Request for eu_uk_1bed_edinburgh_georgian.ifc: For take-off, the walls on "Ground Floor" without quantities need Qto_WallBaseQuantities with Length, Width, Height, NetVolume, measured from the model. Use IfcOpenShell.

First a look at what the model holds.

```python
import ifcopenshell
import ifcopenshell.util.element
import ifcopenshell.util.unit

model = ifcopenshell.open("eu_uk_1bed_edinburgh_georgian.ifc")
print(model.schema)
for unit_type in ("LENGTHUNIT", "AREAUNIT", "VOLUMEUNIT"):
    print(unit_type, ifcopenshell.util.unit.calculate_unit_scale(model, unit_type))
storey = next(s for s in model.by_type("IfcBuildingStorey") if s.Name == "Ground Floor")
walls = [e for e in ifcopenshell.util.element.get_decomposition(storey) if e.is_a("IfcWall")]
for e in sorted(walls, key=lambda e: e.id()):
    print(e.id(), e.is_a(), e.Name, list(ifcopenshell.util.element.get_psets(e, qtos_only=True)), sep=" | ")
```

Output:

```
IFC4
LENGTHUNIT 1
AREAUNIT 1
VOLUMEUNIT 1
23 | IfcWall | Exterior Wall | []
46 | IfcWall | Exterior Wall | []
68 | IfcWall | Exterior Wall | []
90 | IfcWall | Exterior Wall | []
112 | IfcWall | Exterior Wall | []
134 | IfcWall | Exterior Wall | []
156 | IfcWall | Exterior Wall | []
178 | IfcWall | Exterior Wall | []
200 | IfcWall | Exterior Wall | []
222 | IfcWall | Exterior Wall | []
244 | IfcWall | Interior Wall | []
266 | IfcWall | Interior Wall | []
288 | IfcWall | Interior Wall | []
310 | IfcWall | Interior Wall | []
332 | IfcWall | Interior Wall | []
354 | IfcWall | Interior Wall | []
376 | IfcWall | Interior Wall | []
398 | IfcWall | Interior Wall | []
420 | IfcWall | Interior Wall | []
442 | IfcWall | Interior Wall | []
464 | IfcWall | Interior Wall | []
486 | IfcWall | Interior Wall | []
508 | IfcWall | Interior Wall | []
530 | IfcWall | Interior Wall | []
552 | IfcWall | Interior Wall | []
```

```python
import ifcopenshell
import ifcopenshell.api.pset
import ifcopenshell.geom
import ifcopenshell.util.element
import ifcopenshell.util.shape
import ifcopenshell.util.unit

model = ifcopenshell.open("eu_uk_1bed_edinburgh_georgian.ifc")
unit_scale = ifcopenshell.util.unit.calculate_unit_scale(model)
volume_scale = ifcopenshell.util.unit.calculate_unit_scale(model, "VOLUMEUNIT")
settings = ifcopenshell.geom.settings()

storey = next(s for s in model.by_type("IfcBuildingStorey") if s.Name == "Ground Floor")
walls = [e for e in ifcopenshell.util.element.get_decomposition(storey) if e.is_a("IfcWall")]

for e in sorted(walls, key=lambda e: e.id()):
    if ifcopenshell.util.element.get_psets(e, qtos_only=True, should_inherit=False):
        continue
    # Geometry comes back in metres, in the element's own axes.
    shape = ifcopenshell.geom.create_shape(settings, e)
    values = {
        "Length": ifcopenshell.util.shape.get_x(shape.geometry) / unit_scale,
        "Width": ifcopenshell.util.shape.get_y(shape.geometry) / unit_scale,
        "Height": ifcopenshell.util.shape.get_z(shape.geometry) / unit_scale,
        "NetVolume": ifcopenshell.util.shape.get_volume(shape.geometry) / volume_scale,
    }
    qto = ifcopenshell.api.pset.add_qto(model, product=e, name="Qto_WallBaseQuantities")
    ifcopenshell.api.pset.edit_qto(model, qto=qto, properties=values)
    print(e.id(), {k: round(v, 3) for k, v in values.items()})

model.write("eu_uk_1bed_edinburgh_georgian_edited.ifc")
```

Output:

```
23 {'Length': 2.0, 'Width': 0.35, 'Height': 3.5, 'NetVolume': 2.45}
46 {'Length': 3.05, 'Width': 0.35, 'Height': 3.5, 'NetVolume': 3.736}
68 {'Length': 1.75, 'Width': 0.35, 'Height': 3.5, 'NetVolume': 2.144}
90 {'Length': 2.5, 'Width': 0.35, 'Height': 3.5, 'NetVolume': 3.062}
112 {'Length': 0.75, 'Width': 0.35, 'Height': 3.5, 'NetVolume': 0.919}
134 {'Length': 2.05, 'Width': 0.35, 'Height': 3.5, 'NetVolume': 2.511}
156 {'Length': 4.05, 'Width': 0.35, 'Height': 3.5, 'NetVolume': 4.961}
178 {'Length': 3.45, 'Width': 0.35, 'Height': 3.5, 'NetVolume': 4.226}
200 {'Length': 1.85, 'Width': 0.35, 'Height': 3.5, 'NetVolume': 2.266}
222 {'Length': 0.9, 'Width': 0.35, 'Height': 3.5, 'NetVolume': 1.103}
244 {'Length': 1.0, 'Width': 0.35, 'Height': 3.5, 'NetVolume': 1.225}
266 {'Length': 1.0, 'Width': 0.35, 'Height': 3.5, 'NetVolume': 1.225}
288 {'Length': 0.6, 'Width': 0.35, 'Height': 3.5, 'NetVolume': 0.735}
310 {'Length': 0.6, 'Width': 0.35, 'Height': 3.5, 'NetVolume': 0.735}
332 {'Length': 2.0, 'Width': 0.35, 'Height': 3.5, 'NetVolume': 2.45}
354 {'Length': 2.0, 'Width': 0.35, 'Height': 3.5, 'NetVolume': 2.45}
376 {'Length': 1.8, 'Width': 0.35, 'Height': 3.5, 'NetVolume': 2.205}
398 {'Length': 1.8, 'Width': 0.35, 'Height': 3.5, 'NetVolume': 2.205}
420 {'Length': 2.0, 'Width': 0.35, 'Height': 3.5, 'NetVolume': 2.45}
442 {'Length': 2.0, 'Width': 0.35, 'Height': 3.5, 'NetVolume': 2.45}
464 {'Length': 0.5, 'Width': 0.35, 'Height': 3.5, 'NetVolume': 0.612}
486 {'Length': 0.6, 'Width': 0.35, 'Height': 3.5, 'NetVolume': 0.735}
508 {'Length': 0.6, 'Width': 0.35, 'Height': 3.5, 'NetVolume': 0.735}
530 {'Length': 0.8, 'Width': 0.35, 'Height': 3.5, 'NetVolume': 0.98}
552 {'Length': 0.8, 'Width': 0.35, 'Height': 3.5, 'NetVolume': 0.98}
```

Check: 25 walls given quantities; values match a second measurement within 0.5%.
